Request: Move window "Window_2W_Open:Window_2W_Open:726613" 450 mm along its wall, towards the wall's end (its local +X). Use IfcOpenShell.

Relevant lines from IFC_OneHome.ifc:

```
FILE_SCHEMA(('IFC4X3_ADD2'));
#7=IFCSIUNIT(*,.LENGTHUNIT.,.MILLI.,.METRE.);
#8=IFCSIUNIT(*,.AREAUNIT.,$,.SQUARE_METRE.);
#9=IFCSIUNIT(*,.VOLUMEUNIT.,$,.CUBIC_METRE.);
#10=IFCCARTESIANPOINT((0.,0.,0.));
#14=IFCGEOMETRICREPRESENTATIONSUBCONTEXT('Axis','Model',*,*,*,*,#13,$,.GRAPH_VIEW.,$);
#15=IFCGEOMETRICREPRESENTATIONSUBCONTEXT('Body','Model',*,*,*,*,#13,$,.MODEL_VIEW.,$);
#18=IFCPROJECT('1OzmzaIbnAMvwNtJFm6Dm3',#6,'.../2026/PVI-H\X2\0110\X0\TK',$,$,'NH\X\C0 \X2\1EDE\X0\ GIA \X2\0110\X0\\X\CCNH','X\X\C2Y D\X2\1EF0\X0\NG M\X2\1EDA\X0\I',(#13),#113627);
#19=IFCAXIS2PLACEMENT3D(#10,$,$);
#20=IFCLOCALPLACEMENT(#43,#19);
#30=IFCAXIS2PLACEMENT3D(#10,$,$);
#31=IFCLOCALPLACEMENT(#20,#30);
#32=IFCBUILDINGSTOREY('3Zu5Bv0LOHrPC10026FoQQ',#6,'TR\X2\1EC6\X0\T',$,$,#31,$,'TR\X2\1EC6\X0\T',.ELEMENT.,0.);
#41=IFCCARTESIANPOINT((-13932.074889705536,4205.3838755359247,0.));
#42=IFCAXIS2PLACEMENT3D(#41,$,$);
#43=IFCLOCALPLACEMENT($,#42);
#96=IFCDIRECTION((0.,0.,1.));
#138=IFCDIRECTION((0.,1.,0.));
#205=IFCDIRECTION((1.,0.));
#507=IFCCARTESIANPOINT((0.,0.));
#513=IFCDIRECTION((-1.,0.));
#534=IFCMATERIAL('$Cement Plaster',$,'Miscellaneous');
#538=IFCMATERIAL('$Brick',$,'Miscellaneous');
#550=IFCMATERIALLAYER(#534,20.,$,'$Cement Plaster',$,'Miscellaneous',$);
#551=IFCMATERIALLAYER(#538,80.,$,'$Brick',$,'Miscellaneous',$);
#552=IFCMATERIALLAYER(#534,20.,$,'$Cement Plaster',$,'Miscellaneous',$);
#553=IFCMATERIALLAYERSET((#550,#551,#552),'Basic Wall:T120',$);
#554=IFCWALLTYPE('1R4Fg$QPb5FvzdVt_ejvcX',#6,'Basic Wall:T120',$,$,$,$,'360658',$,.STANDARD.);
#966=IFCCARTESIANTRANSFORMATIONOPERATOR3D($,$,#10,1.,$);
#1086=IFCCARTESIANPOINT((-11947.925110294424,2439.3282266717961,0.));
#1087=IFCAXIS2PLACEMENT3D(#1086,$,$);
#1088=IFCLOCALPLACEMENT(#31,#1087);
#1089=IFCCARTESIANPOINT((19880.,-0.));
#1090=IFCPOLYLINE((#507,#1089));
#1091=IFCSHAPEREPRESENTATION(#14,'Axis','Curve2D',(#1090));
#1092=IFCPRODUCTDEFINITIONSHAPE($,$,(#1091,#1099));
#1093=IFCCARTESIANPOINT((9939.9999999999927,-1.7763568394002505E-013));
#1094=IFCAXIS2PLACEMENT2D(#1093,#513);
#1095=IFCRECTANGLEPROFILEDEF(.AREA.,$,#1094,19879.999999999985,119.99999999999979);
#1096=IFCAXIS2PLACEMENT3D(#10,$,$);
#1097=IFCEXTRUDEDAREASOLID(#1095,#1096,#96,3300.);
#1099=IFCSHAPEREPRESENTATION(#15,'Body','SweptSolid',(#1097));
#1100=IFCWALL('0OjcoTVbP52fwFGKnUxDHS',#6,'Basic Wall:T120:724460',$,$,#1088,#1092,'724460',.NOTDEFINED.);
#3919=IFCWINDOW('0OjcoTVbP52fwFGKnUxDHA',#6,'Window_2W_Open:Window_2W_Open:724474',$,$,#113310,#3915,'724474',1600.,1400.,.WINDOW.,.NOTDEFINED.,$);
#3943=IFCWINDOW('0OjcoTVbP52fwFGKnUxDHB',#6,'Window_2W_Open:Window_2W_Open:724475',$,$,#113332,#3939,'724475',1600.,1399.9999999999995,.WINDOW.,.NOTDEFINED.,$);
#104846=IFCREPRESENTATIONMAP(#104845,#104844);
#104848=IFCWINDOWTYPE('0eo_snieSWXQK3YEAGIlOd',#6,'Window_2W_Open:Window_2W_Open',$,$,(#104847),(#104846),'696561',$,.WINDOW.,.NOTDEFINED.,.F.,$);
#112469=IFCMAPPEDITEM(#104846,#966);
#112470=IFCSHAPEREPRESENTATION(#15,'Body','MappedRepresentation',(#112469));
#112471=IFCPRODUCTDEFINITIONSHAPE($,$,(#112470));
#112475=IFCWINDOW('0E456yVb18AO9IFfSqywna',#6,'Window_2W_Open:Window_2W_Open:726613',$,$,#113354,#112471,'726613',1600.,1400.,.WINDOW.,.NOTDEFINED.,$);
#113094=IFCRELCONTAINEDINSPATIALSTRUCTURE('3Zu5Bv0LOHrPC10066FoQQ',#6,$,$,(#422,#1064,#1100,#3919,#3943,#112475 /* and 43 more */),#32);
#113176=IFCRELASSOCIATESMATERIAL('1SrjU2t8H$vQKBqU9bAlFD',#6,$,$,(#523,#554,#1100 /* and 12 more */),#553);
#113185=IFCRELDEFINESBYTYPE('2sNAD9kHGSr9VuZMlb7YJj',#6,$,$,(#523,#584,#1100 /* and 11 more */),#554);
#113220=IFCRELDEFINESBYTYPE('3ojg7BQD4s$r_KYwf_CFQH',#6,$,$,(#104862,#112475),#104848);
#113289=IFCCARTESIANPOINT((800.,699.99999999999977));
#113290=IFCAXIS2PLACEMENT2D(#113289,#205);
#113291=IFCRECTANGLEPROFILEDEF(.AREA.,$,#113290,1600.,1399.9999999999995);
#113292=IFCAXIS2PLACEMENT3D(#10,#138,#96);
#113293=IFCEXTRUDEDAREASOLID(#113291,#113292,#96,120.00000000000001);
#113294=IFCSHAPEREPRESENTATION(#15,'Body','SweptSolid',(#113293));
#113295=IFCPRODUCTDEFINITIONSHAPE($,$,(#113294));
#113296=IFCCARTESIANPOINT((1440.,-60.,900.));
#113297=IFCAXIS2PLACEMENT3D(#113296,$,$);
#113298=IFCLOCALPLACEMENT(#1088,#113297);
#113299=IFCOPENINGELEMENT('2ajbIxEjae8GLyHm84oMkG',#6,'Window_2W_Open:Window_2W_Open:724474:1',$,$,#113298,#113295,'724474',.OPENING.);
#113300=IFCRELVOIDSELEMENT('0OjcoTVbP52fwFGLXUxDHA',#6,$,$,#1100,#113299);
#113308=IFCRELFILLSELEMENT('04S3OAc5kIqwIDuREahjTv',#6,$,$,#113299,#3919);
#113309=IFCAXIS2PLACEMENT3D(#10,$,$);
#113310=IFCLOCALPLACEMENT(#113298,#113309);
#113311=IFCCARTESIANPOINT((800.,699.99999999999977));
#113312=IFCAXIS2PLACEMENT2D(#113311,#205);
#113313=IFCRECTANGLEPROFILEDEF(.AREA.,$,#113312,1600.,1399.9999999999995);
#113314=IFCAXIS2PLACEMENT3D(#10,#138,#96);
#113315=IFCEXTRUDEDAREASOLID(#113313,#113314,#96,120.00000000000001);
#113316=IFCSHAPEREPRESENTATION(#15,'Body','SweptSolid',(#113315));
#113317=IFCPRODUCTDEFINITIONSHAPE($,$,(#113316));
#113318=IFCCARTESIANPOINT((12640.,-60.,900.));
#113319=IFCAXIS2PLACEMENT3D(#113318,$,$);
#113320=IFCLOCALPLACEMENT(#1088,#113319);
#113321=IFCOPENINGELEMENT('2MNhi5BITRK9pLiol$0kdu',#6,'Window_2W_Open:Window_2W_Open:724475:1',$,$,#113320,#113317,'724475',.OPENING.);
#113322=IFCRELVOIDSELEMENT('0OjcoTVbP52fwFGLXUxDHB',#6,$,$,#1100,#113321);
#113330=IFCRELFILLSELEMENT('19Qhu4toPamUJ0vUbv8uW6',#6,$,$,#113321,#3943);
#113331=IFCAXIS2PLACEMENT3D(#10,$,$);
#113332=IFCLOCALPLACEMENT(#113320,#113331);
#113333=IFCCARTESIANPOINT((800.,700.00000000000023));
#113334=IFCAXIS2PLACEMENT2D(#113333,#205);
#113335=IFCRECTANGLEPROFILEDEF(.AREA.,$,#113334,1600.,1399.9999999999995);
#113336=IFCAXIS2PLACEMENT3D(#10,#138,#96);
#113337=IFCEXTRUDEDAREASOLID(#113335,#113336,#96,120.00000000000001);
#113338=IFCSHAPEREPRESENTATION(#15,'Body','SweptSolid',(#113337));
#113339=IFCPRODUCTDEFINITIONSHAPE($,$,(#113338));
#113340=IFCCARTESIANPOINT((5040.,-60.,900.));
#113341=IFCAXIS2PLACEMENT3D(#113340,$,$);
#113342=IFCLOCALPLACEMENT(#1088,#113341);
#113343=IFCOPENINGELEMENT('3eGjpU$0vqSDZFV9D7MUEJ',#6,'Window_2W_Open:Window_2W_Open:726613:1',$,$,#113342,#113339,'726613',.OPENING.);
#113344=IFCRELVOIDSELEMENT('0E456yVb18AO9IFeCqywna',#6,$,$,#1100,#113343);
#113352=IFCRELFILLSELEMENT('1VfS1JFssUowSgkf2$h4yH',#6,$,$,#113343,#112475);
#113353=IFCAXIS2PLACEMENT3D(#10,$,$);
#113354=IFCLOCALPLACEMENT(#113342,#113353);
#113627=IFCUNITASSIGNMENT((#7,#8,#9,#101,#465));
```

```python
import ifcopenshell
import ifcopenshell.api.geometry
import ifcopenshell.util.placement
import ifcopenshell.util.unit

model = ifcopenshell.open("IFC_OneHome.ifc")
unit_scale = ifcopenshell.util.unit.calculate_unit_scale(model)

window = model.by_guid("0E456yVb18AO9IFfSqywna")
opening = window.FillsVoids[0].RelatingOpeningElement
wall = opening.VoidsElements[0].RelatingBuildingElement

wall_matrix = ifcopenshell.util.placement.get_local_placement(wall.ObjectPlacement)
shift = wall_matrix[:3, 0] * 0.45 / unit_scale
before = ifcopenshell.util.placement.get_local_placement(window.ObjectPlacement)[:3, 3].copy()

# The window is placed relative to its opening, so it follows when the opening moves.
matrix = ifcopenshell.util.placement.get_local_placement(opening.ObjectPlacement)
matrix[:3, 3] += shift
ifcopenshell.api.geometry.edit_object_placement(
    model, product=opening, matrix=matrix, is_si=False, should_transform_children=True
)

after = ifcopenshell.util.placement.get_local_placement(window.ObjectPlacement)[:3, 3]
print("window moved by", (after - before).round(3) + 0.0)

model.write("IFC_OneHome_rev.ifc")
```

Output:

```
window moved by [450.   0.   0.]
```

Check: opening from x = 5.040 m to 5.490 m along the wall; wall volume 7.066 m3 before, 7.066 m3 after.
